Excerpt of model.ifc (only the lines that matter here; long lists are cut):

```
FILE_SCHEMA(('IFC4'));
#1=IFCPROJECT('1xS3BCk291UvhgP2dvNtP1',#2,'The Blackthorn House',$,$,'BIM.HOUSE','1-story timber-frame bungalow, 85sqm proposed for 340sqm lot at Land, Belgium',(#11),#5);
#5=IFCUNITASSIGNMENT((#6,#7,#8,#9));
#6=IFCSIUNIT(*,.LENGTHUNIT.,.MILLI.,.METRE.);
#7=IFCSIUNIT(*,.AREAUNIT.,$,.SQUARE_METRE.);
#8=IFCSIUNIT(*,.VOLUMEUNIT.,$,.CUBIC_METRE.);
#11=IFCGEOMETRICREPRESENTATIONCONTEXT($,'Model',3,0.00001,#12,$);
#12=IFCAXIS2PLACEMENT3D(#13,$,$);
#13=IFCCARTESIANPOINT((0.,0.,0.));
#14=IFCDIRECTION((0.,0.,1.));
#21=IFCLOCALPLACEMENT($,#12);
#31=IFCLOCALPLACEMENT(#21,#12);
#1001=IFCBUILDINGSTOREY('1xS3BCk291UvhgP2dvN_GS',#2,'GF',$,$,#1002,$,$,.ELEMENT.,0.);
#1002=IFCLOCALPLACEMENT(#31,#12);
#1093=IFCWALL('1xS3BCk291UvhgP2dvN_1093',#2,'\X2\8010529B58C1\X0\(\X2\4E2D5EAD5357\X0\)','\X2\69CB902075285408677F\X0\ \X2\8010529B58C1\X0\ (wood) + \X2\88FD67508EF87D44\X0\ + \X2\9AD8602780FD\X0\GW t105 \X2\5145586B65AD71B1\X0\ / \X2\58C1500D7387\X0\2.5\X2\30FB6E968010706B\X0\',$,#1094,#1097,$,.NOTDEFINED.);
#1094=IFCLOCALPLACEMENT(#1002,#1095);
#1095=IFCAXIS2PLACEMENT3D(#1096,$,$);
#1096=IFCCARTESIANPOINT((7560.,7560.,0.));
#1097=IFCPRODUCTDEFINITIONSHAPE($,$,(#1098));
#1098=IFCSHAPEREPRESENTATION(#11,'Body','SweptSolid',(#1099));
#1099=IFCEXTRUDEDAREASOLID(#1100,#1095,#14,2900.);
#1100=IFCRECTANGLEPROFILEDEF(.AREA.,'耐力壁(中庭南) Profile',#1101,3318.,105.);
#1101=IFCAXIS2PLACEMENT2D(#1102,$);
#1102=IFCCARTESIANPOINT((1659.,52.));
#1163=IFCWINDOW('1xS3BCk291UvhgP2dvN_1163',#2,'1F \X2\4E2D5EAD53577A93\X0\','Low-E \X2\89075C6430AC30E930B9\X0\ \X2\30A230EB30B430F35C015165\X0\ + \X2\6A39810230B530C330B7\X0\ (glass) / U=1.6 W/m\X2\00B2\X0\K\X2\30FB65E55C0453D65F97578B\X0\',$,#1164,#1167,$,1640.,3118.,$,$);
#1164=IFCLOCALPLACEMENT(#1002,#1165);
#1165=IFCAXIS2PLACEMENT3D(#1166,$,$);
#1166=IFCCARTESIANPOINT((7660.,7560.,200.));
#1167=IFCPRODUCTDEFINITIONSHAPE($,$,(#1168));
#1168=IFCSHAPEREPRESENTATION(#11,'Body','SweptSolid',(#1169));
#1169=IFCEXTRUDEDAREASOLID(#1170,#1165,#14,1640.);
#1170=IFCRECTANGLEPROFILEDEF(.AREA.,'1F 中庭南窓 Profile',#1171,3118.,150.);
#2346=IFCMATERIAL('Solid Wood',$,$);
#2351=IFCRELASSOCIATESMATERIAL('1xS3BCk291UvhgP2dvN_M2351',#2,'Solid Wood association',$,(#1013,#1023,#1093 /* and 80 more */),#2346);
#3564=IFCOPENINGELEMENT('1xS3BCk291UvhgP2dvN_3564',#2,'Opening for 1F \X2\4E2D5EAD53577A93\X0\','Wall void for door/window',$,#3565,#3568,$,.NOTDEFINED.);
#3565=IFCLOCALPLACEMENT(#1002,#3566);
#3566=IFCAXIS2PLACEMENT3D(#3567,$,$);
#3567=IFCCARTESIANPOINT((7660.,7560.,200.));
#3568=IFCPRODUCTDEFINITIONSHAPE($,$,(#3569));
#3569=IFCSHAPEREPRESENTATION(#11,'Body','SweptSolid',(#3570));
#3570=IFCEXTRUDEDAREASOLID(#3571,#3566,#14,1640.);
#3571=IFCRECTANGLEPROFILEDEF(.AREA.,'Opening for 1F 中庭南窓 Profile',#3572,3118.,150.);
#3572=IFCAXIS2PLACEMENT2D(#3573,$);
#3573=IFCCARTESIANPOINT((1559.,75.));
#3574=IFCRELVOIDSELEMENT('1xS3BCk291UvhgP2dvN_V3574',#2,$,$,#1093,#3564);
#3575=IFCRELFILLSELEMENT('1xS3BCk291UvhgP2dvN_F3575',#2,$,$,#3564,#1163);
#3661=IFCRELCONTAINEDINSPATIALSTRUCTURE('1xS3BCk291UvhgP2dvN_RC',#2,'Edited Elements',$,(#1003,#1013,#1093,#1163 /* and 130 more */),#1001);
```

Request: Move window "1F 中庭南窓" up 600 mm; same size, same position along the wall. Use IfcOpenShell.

```python
import numpy as np
import ifcopenshell
import ifcopenshell.api.geometry
import ifcopenshell.util.placement
import ifcopenshell.util.unit

model = ifcopenshell.open("model.ifc")
unit_scale = ifcopenshell.util.unit.calculate_unit_scale(model)

window = model.by_id(1163)
opening = window.FillsVoids[0].RelatingOpeningElement
dz = 0.6 / unit_scale

shift = np.array([0.0, 0.0, dz])
# The window is not placed relative to its opening, so move both.
for product in (opening, window):
    matrix = ifcopenshell.util.placement.get_local_placement(product.ObjectPlacement)
    matrix[:3, 3] += shift
    ifcopenshell.api.geometry.edit_object_placement(model, product=product, matrix=matrix, is_si=False)

print(f"moved by {dz * unit_scale:+.3f} m")

model.write("model_updated.ifc")
```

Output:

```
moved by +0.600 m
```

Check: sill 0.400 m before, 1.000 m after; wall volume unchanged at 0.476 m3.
